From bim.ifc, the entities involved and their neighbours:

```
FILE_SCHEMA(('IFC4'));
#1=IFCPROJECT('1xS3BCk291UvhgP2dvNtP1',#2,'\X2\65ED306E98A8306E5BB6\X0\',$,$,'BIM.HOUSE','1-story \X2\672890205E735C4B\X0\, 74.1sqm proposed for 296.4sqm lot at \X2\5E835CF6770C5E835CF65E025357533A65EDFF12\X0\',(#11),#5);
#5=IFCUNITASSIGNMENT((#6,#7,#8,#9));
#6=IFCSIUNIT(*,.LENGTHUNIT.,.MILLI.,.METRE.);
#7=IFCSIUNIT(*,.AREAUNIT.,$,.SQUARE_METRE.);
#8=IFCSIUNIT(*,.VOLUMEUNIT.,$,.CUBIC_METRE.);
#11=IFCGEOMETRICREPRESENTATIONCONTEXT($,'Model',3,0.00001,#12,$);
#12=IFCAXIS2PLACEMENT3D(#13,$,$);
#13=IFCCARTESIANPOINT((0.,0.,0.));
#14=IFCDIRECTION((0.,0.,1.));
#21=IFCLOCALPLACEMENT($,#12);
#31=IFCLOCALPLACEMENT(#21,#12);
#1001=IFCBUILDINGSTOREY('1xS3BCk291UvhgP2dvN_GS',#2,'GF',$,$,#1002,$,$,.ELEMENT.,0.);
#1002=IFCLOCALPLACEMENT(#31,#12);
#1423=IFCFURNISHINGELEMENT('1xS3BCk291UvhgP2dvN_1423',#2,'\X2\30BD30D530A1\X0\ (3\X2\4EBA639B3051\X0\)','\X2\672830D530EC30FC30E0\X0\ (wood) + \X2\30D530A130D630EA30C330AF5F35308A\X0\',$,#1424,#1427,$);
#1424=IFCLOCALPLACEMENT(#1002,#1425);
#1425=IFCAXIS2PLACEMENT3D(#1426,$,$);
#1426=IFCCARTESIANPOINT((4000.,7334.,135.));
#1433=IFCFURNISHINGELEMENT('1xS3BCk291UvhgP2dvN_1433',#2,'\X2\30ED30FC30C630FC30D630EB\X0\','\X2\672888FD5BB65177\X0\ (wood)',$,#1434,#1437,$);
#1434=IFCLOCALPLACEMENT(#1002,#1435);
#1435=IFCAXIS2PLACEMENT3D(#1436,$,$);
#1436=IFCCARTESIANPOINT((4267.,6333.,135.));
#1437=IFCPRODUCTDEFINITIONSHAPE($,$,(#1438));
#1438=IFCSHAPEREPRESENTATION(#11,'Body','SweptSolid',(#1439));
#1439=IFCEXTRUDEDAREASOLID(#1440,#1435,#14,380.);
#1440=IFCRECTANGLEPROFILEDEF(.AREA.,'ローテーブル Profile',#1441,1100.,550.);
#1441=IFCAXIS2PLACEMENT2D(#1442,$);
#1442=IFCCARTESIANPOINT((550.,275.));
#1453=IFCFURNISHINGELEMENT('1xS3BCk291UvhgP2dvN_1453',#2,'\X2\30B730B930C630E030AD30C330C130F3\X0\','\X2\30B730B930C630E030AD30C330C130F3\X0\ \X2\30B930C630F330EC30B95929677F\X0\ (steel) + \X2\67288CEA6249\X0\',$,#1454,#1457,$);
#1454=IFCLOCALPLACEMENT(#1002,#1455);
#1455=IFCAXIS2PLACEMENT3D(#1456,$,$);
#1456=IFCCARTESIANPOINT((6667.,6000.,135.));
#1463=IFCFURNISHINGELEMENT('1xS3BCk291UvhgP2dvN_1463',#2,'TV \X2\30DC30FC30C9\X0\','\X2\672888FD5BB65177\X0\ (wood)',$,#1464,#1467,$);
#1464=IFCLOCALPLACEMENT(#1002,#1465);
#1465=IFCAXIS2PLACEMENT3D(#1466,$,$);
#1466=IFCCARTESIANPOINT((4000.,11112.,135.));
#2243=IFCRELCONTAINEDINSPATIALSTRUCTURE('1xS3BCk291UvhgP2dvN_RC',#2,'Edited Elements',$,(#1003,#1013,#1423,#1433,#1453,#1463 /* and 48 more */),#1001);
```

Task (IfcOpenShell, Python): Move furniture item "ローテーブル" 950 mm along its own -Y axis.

```python
import ifcopenshell
import ifcopenshell.api.geometry
import ifcopenshell.util.placement

model = ifcopenshell.open("bim.ifc")

item = model.by_id(1433)
matrix = ifcopenshell.util.placement.get_local_placement(item.ObjectPlacement)
matrix[:3, 3] -= matrix[:3, 1] * 950.0
ifcopenshell.api.geometry.edit_object_placement(model, product=item, matrix=matrix, is_si=False)

print(ifcopenshell.util.placement.get_local_placement(item.ObjectPlacement).round(3) + 0.0)

model.write("bim_updated.ifc")
```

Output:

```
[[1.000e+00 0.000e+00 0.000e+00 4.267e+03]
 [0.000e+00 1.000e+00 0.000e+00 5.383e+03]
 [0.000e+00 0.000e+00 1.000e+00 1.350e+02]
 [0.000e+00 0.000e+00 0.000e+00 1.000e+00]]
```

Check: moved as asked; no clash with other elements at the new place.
